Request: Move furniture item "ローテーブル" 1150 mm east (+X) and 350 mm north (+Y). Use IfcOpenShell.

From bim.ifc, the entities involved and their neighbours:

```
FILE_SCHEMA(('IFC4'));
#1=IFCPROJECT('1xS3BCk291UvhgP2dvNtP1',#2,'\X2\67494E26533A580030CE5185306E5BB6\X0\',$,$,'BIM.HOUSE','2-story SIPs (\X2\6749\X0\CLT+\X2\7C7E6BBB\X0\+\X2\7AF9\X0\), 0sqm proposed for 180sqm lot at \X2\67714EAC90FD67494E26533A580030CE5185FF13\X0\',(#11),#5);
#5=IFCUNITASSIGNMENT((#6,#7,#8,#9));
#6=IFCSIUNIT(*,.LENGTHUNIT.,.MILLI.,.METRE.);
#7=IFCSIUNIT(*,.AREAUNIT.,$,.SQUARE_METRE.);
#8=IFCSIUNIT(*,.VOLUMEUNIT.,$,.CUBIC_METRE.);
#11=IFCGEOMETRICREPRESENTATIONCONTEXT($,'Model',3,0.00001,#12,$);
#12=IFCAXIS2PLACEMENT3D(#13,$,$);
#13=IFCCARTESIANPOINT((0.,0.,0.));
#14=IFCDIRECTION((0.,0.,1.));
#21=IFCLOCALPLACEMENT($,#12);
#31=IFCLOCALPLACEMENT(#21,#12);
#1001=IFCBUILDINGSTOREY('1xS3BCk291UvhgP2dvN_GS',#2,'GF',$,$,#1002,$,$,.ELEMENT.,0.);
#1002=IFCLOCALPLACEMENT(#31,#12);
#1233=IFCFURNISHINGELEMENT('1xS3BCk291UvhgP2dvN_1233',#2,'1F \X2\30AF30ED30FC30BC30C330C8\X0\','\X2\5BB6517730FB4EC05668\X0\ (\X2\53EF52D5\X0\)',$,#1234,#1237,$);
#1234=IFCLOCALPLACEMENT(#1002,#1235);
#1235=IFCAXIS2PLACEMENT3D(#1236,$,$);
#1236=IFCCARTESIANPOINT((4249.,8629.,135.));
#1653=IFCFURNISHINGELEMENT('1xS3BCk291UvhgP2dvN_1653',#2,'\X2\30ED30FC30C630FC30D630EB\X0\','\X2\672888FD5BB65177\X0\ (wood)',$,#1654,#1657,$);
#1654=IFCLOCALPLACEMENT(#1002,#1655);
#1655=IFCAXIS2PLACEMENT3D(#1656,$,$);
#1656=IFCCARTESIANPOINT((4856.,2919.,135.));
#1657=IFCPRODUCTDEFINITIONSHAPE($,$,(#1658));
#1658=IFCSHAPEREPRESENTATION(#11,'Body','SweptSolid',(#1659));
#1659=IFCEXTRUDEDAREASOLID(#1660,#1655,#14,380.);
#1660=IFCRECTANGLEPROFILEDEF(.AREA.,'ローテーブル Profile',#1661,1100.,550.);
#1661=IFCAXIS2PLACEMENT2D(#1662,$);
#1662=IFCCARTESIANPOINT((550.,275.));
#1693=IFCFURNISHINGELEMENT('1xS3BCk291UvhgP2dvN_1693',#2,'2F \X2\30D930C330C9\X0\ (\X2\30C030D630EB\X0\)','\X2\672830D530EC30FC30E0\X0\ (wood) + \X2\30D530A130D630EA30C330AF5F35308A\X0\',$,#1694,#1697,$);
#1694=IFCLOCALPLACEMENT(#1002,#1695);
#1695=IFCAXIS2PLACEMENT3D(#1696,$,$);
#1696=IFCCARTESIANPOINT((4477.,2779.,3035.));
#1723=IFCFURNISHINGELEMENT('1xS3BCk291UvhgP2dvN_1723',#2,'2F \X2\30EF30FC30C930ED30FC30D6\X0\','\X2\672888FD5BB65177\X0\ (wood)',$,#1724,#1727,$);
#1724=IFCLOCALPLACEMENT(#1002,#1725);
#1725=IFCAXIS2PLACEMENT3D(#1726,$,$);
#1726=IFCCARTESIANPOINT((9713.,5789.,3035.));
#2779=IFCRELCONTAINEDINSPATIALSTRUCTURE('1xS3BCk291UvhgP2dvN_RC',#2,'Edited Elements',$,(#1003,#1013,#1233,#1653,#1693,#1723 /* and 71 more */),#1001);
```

```python
import ifcopenshell
import ifcopenshell.api.geometry
import ifcopenshell.util.placement
import ifcopenshell.util.unit

model = ifcopenshell.open("bim.ifc")
unit_scale = ifcopenshell.util.unit.calculate_unit_scale(model)

item = model.by_id(1653)
matrix = ifcopenshell.util.placement.get_local_placement(item.ObjectPlacement)
matrix[0, 3] += 1.15 / unit_scale
matrix[1, 3] += 0.35 / unit_scale
ifcopenshell.api.geometry.edit_object_placement(model, product=item, matrix=matrix, is_si=False)

print(ifcopenshell.util.placement.get_local_placement(item.ObjectPlacement).round(3) + 0.0)

model.write("bim_v2.ifc")
```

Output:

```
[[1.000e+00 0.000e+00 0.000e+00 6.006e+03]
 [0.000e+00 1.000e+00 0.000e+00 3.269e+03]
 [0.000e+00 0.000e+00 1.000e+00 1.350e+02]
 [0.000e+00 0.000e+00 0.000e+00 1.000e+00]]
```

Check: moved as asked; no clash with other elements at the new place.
